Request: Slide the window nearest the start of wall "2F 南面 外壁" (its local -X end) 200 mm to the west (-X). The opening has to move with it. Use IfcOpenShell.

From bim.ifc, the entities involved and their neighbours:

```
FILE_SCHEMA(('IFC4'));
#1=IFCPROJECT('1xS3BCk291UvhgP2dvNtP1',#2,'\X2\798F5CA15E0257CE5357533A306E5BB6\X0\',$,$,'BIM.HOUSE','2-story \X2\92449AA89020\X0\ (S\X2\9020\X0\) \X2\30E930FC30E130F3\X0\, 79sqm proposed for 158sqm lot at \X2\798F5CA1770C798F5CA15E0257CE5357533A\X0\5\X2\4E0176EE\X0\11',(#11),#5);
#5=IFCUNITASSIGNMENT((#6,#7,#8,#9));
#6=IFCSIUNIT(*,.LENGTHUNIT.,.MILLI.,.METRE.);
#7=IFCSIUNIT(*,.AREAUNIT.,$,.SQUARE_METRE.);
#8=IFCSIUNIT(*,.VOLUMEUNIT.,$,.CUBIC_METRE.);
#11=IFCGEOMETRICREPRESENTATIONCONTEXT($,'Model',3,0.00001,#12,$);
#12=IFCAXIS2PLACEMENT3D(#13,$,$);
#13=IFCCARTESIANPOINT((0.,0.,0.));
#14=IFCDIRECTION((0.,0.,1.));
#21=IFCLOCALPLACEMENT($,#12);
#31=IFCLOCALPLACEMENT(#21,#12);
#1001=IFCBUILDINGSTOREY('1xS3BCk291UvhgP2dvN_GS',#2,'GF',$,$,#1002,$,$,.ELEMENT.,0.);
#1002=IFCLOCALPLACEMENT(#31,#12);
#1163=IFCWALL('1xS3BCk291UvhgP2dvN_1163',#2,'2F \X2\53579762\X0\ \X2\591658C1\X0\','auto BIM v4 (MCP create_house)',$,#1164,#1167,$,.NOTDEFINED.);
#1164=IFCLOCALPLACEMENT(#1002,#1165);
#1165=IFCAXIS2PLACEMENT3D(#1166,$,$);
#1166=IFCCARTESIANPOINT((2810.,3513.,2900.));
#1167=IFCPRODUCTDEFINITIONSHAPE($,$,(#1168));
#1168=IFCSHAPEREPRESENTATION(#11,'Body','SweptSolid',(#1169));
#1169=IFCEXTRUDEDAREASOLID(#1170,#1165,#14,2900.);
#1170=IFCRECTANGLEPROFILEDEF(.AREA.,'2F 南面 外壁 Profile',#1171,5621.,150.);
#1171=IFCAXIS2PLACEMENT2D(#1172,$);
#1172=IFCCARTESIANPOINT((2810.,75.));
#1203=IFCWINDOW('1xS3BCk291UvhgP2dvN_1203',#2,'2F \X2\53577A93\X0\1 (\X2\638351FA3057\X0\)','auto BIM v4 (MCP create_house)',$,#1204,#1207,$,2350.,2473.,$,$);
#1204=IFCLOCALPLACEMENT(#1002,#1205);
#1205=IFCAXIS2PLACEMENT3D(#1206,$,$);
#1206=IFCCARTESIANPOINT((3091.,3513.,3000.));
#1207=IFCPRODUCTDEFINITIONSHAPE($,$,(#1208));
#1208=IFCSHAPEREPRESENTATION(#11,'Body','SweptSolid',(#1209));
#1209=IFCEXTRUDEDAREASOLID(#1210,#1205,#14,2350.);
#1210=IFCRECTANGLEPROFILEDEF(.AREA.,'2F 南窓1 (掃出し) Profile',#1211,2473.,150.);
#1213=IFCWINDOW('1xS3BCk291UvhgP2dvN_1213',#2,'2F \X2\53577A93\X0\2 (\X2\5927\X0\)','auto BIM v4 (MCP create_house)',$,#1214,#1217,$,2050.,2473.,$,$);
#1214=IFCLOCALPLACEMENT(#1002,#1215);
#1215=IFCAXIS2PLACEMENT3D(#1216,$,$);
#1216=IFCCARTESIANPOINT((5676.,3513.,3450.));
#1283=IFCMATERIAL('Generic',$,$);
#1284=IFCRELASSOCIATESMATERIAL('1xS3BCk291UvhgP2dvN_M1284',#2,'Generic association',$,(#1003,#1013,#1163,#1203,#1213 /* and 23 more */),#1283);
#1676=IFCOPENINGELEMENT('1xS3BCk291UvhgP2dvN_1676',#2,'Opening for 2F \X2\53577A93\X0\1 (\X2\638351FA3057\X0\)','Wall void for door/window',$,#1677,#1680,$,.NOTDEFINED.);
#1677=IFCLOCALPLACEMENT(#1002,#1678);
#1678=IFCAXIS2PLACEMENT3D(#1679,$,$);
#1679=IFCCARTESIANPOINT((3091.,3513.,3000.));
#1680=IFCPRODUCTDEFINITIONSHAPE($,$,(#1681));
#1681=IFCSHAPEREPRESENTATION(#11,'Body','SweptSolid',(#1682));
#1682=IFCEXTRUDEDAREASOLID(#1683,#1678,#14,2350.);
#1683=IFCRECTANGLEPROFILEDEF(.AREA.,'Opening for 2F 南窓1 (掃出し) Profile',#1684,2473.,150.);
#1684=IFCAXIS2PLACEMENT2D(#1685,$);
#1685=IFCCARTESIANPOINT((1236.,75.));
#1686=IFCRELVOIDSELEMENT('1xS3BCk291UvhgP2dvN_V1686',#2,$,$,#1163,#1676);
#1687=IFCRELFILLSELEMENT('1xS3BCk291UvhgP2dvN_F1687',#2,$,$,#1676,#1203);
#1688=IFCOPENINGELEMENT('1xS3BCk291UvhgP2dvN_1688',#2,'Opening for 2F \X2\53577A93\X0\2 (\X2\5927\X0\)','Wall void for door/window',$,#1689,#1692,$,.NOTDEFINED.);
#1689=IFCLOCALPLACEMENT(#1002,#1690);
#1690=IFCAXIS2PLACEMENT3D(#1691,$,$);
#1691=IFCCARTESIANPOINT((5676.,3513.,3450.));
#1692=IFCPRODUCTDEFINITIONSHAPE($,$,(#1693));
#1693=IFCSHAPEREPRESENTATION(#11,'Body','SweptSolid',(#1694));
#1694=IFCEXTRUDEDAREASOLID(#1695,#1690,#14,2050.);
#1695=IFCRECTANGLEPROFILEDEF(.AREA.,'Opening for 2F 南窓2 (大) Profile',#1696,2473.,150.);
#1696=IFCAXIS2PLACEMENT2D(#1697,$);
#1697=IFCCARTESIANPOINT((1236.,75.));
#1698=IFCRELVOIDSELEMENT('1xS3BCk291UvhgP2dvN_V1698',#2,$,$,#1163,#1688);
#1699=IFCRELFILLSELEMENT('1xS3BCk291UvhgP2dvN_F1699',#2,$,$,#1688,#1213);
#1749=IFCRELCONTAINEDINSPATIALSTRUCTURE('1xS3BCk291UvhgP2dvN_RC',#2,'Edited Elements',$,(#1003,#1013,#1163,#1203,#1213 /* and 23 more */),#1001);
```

```python
import ifcopenshell
import ifcopenshell.api.geometry
import ifcopenshell.util.placement

model = ifcopenshell.open("bim.ifc")

window = model.by_guid("1xS3BCk291UvhgP2dvN_1203")
opening = window.FillsVoids[0].RelatingOpeningElement
wall = opening.VoidsElements[0].RelatingBuildingElement

wall_matrix = ifcopenshell.util.placement.get_local_placement(wall.ObjectPlacement)
shift = wall_matrix[:3, 0] * -200.0
before = ifcopenshell.util.placement.get_local_placement(window.ObjectPlacement)[:3, 3].copy()

# The window is not placed relative to its opening, so move both.
for product in (opening, window):
    matrix = ifcopenshell.util.placement.get_local_placement(product.ObjectPlacement)
    matrix[:3, 3] += shift
    ifcopenshell.api.geometry.edit_object_placement(model, product=product, matrix=matrix, is_si=False)

after = ifcopenshell.util.placement.get_local_placement(window.ObjectPlacement)[:3, 3]
print("window moved by", (after - before).round(3) + 0.0)

model.write("bim_edited.ifc")
```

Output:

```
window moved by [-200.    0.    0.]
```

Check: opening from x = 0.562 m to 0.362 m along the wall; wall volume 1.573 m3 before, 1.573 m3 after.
